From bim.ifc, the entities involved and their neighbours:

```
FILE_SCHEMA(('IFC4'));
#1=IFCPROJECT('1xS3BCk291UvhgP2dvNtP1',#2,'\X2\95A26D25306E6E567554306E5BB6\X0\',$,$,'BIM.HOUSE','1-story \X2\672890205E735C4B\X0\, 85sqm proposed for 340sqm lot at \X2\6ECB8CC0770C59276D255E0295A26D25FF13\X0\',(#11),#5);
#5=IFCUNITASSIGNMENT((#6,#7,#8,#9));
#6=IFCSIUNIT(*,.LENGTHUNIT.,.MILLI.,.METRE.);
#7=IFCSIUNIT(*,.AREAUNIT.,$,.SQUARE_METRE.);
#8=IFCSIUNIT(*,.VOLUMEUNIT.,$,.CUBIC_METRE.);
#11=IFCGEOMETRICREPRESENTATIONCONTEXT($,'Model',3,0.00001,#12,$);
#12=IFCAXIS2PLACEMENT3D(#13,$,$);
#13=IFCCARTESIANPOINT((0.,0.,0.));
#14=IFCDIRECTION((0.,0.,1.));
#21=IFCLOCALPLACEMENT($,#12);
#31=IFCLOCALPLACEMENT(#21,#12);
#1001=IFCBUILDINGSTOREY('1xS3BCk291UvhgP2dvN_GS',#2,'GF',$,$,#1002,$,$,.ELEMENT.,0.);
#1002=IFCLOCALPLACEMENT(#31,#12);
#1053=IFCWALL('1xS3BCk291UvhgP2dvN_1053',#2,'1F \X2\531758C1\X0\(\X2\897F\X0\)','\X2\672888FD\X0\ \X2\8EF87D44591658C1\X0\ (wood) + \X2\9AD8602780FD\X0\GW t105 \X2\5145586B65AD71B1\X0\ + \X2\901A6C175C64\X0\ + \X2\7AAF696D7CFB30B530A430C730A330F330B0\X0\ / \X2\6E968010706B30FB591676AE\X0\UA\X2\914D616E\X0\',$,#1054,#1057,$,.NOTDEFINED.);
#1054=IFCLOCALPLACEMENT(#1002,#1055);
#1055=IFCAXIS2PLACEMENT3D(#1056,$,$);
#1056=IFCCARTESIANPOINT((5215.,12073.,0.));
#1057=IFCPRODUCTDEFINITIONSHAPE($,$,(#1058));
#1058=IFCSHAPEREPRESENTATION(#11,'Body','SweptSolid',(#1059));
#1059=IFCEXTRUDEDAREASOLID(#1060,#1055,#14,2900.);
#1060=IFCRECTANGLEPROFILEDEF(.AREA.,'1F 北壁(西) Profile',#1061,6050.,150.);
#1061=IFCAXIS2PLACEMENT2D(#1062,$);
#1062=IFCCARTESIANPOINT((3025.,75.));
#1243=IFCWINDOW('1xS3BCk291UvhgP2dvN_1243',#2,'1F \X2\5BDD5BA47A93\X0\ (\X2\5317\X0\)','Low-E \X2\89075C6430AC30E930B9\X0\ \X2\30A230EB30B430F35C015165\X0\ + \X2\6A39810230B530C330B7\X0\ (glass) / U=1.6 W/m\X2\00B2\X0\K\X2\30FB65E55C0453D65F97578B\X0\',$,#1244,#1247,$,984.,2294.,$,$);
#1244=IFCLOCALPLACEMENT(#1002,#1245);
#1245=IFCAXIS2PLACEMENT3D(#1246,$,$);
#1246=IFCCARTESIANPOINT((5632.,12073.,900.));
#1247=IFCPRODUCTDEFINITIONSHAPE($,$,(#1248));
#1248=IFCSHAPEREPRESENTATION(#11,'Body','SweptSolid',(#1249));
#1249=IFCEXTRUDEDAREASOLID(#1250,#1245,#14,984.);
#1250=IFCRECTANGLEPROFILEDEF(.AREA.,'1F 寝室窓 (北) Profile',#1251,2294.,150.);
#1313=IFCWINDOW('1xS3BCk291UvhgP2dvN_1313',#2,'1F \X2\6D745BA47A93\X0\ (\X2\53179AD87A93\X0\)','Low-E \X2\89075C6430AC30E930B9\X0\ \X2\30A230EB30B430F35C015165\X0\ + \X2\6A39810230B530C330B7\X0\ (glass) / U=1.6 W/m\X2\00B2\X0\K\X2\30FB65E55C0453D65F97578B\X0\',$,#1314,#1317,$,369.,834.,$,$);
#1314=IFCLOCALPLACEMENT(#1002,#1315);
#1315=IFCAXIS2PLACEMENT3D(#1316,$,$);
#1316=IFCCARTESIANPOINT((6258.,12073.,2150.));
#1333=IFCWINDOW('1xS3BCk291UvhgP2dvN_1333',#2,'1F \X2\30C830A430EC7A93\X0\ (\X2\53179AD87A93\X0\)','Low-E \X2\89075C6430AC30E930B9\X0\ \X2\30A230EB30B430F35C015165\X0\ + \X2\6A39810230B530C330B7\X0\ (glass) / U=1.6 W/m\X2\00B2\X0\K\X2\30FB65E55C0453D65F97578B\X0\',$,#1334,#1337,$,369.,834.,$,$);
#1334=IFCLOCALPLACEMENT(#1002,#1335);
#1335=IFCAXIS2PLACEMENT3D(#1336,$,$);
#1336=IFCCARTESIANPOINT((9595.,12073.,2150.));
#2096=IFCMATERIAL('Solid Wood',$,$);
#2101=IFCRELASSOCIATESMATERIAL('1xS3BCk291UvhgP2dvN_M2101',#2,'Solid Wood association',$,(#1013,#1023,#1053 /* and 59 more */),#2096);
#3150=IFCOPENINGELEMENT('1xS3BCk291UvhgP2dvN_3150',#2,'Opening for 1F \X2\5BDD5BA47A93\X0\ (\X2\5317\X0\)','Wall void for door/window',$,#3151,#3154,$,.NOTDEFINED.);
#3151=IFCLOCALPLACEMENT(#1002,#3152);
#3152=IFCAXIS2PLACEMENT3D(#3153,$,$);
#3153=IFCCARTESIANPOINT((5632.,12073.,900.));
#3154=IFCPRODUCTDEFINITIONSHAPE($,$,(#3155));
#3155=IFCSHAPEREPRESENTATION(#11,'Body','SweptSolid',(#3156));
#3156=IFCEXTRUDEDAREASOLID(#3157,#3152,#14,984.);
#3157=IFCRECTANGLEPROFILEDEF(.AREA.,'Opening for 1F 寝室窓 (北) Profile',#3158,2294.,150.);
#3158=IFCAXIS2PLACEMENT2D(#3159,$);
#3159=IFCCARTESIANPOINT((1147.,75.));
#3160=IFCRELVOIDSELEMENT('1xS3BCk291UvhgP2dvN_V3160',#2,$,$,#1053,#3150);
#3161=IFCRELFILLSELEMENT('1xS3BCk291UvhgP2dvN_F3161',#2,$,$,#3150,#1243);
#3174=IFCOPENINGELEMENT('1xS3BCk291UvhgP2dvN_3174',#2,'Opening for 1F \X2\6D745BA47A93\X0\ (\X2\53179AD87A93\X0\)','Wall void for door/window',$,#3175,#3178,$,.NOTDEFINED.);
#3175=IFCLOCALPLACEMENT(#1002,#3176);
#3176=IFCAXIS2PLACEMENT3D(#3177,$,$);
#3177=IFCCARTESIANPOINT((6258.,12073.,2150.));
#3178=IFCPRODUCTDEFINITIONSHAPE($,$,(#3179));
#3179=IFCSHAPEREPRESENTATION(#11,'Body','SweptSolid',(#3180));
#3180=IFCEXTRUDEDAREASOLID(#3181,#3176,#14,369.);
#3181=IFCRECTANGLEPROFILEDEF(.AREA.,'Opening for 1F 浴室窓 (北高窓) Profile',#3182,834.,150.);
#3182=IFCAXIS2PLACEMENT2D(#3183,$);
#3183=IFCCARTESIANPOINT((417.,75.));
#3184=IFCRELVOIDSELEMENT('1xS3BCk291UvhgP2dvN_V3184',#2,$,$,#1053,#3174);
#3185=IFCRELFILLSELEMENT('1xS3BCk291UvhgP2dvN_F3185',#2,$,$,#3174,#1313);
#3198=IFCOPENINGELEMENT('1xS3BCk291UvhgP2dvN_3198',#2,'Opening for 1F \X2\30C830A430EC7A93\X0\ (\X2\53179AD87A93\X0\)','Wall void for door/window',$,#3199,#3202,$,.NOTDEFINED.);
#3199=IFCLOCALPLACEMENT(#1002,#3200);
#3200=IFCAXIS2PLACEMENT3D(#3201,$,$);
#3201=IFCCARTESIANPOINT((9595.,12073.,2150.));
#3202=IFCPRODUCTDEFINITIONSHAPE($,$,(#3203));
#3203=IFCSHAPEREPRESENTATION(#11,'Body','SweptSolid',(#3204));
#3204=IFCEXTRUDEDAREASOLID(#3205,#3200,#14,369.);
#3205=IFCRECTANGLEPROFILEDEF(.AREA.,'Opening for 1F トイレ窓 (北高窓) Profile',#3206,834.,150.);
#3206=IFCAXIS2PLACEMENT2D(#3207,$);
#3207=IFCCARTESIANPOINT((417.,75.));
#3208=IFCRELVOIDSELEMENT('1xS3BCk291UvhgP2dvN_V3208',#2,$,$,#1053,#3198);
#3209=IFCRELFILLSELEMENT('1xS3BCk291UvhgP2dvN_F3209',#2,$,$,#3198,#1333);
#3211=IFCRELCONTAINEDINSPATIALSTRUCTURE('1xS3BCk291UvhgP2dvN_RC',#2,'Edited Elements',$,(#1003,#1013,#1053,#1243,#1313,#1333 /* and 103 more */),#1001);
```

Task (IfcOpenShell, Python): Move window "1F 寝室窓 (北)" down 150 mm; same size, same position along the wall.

```python
import numpy as np
import ifcopenshell
import ifcopenshell.api.geometry
import ifcopenshell.util.placement
import ifcopenshell.util.unit

model = ifcopenshell.open("bim.ifc")
unit_scale = ifcopenshell.util.unit.calculate_unit_scale(model)

window = model.by_guid("1xS3BCk291UvhgP2dvN_1243")
opening = window.FillsVoids[0].RelatingOpeningElement
dz = -0.15 / unit_scale

shift = np.array([0.0, 0.0, dz])
# The window is not placed relative to its opening, so move both.
for product in (opening, window):
    matrix = ifcopenshell.util.placement.get_local_placement(product.ObjectPlacement)
    matrix[:3, 3] += shift
    ifcopenshell.api.geometry.edit_object_placement(model, product=product, matrix=matrix, is_si=False)

print(f"moved by {dz * unit_scale:+.3f} m")

model.write("bim-out.ifc")
```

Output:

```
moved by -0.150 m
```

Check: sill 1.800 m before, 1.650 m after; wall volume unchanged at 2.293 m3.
